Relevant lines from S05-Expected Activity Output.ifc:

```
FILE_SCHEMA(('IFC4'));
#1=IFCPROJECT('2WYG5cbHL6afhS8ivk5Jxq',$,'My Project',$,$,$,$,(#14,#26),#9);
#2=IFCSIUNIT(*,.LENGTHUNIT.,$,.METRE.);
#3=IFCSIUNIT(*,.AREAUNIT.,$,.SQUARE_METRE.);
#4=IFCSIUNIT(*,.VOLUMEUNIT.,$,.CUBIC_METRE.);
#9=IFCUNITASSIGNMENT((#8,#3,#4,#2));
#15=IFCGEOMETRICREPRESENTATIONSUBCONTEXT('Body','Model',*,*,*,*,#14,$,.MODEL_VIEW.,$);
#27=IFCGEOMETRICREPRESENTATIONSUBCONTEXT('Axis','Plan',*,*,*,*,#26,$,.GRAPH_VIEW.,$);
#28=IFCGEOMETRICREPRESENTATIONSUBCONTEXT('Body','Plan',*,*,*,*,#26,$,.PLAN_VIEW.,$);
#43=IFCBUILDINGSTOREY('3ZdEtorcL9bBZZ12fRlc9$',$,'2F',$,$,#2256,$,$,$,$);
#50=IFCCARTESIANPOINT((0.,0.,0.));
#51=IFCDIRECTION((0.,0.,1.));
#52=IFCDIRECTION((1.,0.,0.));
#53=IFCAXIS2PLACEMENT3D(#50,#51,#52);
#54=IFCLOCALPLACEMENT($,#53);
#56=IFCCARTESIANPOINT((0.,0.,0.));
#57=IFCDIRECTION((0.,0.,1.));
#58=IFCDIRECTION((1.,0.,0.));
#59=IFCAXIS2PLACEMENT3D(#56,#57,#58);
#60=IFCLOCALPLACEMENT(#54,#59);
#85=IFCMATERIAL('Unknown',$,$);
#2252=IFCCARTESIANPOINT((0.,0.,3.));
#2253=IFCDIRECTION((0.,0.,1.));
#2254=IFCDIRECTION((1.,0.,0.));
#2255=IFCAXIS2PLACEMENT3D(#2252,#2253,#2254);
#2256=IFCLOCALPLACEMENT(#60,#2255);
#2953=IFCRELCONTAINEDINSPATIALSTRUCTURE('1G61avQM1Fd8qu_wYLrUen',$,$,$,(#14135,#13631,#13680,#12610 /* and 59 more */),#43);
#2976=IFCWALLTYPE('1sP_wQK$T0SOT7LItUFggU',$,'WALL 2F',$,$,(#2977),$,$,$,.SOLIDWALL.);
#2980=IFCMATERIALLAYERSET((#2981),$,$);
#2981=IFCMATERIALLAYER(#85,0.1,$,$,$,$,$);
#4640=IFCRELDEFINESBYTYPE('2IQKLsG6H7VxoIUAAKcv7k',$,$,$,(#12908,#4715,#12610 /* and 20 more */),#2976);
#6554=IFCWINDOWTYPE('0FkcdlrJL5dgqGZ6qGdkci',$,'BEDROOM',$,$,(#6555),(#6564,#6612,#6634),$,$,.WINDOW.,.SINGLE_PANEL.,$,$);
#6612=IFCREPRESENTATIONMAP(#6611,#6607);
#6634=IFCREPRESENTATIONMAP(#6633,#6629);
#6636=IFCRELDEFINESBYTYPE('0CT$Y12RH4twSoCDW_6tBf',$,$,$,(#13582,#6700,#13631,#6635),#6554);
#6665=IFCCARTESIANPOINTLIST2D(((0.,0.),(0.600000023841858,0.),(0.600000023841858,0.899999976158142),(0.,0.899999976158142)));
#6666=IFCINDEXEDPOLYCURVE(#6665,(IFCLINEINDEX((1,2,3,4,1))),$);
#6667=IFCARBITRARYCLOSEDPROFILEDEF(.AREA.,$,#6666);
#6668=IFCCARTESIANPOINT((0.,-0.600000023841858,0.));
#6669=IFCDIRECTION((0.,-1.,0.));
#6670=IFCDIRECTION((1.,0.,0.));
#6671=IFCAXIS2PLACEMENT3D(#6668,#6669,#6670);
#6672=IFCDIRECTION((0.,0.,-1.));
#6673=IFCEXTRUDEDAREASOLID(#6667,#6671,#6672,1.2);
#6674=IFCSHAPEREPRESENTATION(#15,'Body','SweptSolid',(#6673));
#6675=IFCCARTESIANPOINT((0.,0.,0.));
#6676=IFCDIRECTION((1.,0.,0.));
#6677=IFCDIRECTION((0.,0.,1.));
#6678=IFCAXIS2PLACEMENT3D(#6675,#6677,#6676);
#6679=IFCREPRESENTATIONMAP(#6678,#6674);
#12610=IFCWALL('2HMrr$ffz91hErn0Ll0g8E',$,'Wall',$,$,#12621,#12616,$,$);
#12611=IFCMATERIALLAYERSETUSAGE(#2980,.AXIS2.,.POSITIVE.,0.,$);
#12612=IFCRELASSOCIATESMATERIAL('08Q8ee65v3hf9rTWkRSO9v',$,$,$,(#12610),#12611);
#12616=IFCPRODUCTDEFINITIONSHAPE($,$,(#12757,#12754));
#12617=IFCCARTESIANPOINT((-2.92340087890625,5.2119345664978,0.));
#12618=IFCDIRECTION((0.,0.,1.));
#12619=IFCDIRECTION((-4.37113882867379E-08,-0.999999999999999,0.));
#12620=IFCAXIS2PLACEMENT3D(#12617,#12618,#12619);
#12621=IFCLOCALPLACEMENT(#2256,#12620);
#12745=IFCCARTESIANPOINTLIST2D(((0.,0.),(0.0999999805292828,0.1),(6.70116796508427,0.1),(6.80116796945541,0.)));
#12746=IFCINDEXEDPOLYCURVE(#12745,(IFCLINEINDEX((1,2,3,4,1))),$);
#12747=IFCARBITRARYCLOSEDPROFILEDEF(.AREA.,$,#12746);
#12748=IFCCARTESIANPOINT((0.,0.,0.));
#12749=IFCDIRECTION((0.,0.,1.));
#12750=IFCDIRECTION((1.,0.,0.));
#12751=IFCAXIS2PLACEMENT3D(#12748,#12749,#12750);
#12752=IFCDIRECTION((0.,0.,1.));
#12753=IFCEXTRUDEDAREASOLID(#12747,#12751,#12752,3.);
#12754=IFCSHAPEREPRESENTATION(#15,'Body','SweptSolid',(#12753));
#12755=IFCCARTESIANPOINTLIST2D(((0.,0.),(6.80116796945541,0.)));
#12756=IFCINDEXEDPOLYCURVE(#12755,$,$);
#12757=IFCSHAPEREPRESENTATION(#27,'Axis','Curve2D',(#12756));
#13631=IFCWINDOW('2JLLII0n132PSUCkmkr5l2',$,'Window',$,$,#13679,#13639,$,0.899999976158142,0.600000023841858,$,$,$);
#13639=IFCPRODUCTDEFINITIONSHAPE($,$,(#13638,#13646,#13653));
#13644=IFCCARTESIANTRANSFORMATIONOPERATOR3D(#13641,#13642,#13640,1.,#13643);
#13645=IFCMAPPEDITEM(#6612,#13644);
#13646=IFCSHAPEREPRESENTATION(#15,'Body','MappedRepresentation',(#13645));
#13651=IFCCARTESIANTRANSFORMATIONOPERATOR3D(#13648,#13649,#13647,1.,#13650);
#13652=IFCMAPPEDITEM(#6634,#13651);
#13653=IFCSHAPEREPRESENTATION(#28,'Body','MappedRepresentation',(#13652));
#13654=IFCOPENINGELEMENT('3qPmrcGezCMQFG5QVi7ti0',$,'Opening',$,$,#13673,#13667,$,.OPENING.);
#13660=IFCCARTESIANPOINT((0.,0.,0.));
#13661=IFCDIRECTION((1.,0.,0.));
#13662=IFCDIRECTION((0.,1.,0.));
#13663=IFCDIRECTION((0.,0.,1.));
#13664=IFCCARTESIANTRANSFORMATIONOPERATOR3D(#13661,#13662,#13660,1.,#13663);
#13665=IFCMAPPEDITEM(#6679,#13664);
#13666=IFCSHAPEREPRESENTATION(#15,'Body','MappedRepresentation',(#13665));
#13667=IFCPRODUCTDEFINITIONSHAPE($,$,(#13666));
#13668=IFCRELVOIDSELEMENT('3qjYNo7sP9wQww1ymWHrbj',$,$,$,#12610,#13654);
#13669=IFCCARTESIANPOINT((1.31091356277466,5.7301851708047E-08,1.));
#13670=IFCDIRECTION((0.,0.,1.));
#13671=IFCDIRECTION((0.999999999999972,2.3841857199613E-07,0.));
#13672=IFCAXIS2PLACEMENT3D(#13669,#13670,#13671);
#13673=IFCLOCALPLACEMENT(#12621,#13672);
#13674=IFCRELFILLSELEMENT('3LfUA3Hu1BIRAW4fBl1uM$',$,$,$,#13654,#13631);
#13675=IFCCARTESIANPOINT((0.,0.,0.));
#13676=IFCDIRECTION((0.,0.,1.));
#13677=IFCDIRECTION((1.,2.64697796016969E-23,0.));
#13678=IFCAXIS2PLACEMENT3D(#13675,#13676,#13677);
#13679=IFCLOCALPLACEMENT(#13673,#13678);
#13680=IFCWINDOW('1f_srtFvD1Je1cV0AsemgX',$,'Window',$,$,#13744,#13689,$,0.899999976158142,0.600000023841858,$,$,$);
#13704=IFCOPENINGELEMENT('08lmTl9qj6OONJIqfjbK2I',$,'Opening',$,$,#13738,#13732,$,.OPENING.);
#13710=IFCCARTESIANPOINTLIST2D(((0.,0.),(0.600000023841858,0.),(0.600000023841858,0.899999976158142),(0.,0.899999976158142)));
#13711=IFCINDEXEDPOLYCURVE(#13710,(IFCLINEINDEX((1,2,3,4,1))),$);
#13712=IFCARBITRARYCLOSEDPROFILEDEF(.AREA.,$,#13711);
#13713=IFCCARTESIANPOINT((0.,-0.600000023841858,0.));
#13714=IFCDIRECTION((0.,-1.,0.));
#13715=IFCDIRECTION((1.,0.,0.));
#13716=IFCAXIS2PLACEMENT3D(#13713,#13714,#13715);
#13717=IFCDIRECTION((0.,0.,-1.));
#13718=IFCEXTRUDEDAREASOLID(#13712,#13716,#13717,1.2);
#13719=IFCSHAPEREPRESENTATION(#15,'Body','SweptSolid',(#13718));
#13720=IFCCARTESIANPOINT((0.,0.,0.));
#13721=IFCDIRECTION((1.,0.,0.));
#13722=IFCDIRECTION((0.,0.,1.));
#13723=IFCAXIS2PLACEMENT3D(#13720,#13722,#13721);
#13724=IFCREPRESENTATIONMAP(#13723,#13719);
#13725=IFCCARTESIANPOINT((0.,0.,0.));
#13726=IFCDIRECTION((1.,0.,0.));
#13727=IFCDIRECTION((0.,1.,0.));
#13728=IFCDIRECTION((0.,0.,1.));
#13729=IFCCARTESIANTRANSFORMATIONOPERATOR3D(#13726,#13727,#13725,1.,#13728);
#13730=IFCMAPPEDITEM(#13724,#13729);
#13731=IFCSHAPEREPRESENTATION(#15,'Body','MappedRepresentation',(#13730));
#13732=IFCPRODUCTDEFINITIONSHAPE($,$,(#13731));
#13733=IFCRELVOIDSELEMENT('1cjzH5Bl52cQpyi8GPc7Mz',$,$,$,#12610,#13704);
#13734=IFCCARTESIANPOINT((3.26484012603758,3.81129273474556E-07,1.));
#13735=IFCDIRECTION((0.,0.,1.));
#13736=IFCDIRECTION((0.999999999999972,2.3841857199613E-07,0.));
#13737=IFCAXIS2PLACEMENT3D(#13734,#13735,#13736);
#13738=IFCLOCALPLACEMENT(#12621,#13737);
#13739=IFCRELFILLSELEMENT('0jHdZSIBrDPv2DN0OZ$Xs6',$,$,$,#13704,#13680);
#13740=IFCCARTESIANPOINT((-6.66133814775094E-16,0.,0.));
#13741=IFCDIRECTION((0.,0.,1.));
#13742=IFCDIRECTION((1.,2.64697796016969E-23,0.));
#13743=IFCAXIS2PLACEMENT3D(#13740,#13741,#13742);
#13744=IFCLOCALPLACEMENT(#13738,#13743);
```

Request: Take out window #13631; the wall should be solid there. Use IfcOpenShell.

```python
import ifcopenshell
import ifcopenshell.api.feature
import ifcopenshell.api.root
import ifcopenshell.geom
import ifcopenshell.util.shape

model = ifcopenshell.open("S05-Expected Activity Output.ifc")
settings = ifcopenshell.geom.settings()


def volume(element):
    """Net volume in cubic metres, openings subtracted."""
    shape = ifcopenshell.geom.create_shape(settings, element)
    return ifcopenshell.util.shape.get_volume(shape.geometry)


window = model.by_id(13631)
opening = window.FillsVoids[0].RelatingOpeningElement
wall = opening.VoidsElements[0].RelatingBuildingElement
before = volume(wall)

ifcopenshell.api.root.remove_product(model, product=window)
ifcopenshell.api.feature.remove_feature(model, feature=opening)

after = volume(wall)

print(f"wall volume {before:.3f} -> {after:.3f} m3")

model.write("S05-Expected Activity Output_edited.ifc")
```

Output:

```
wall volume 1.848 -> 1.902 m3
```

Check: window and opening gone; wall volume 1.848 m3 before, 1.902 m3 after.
